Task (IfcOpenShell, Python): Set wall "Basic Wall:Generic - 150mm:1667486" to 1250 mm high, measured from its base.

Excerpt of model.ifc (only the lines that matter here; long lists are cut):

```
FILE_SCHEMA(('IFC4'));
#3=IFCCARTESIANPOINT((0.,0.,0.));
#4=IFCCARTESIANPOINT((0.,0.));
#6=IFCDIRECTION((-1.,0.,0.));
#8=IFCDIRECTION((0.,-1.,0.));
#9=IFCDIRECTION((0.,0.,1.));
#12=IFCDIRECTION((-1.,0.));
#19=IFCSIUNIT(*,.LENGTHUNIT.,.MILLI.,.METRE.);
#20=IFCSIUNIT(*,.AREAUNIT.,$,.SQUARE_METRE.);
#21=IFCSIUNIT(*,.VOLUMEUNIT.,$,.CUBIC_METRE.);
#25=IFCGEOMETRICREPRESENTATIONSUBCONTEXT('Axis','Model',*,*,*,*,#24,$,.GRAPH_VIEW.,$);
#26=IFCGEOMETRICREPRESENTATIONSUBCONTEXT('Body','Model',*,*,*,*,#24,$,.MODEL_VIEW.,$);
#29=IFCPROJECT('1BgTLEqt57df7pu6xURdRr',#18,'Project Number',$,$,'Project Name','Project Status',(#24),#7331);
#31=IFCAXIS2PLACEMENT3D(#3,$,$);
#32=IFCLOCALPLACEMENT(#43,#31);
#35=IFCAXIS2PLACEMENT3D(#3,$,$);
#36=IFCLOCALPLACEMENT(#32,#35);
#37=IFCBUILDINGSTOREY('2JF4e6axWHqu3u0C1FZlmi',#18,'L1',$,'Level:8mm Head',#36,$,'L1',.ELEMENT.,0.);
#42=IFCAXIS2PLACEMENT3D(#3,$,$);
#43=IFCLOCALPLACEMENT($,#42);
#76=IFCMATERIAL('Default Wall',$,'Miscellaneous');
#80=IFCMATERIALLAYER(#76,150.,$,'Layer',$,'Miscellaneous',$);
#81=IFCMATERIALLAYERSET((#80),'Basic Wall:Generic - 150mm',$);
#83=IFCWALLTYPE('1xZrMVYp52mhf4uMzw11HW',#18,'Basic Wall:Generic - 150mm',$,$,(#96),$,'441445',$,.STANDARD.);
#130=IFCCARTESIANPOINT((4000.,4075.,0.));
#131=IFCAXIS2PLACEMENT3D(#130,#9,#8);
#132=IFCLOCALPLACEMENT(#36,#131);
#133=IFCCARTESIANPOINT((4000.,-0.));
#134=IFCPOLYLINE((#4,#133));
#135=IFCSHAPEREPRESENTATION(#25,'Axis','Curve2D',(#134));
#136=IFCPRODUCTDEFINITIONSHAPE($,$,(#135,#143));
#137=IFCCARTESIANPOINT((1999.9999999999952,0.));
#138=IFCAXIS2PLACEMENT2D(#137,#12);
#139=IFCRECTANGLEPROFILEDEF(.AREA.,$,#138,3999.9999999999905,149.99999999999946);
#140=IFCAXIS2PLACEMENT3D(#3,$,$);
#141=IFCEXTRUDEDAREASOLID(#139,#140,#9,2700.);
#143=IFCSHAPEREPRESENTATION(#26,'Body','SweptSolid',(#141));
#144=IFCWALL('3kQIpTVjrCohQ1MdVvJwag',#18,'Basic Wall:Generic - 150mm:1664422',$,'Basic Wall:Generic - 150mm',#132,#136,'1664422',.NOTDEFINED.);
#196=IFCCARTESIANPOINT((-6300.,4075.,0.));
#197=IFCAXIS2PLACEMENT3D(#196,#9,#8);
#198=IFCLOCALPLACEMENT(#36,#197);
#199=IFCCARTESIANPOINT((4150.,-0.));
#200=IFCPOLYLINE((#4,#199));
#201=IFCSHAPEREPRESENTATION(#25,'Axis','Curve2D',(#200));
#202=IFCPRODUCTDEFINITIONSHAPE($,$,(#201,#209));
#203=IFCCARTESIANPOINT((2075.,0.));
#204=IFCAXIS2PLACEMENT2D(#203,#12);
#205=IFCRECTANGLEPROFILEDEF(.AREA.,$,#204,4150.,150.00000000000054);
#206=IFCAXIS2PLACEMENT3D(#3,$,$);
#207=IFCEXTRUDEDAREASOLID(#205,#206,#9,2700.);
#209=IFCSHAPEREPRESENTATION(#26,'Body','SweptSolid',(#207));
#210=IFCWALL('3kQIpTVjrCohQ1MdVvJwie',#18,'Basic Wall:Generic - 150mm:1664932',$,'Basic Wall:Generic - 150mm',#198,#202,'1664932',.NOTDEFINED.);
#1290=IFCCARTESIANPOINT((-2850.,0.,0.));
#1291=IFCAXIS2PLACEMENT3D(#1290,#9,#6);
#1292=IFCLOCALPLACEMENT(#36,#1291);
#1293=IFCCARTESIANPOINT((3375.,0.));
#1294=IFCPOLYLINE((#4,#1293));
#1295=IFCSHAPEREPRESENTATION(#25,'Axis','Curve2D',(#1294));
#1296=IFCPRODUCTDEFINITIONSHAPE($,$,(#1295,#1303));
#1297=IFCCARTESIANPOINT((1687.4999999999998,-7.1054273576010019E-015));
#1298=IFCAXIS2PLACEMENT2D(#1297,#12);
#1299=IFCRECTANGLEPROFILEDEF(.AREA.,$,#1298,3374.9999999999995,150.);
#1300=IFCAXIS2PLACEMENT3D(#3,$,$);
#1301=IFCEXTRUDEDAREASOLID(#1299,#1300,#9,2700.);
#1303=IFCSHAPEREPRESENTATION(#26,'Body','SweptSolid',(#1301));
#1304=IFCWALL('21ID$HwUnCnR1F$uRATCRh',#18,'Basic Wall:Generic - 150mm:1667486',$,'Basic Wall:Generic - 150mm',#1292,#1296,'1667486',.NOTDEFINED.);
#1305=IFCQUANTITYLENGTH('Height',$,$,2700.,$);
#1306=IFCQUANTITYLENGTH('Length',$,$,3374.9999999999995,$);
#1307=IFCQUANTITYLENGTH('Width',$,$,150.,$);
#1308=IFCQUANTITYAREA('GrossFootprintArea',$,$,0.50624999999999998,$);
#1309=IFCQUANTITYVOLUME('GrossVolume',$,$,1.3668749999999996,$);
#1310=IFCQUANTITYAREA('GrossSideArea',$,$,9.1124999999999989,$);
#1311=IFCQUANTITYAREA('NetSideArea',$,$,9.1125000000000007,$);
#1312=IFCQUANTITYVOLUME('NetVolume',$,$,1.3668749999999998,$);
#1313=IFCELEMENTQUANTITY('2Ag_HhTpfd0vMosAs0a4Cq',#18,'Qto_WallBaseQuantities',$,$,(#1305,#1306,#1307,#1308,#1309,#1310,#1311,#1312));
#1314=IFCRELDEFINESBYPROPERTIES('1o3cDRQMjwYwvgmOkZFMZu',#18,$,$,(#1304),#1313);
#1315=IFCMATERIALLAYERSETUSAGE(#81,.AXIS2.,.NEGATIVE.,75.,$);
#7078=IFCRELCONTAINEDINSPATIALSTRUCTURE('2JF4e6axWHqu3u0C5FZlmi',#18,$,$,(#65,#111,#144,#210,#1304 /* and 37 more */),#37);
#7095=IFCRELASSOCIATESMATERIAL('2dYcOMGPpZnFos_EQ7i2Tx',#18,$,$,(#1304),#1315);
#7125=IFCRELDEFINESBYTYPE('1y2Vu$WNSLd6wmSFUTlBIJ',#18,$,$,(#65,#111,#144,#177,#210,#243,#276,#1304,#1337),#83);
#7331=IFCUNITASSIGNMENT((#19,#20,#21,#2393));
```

```python
import ifcopenshell
import ifcopenshell.api.pset
import ifcopenshell.geom
import ifcopenshell.util.element
import ifcopenshell.util.representation
import ifcopenshell.util.shape
import ifcopenshell.util.unit

model = ifcopenshell.open("model.ifc")
unit_scale = ifcopenshell.util.unit.calculate_unit_scale(model)
area_scale = ifcopenshell.util.unit.calculate_unit_scale(model, "AREAUNIT")
volume_scale = ifcopenshell.util.unit.calculate_unit_scale(model, "VOLUMEUNIT")
settings = ifcopenshell.geom.settings()


def volume(element):
    """Net volume in cubic metres, openings subtracted."""
    shape = ifcopenshell.geom.create_shape(settings, element)
    return ifcopenshell.util.shape.get_volume(shape.geometry)


wall = model.by_guid("21ID$HwUnCnR1F$uRATCRh")
before = volume(wall)

body = ifcopenshell.util.representation.get_representation(wall, "Model", "Body")
solid = body.Items[0]
old_height = solid.Depth
solid.Depth = 1250.0
after = volume(wall)
thickness = 0.15  # wall thickness in metres

# Update the stored height, areas and volumes.
qto = model.by_id(ifcopenshell.util.element.get_pset(wall, "Qto_WallBaseQuantities", should_inherit=False)["id"])
ifcopenshell.api.pset.edit_qto(model, qto=qto, properties={
    "Height": solid.Depth,
    "GrossVolume": ifcopenshell.util.element.get_pset(wall, "Qto_WallBaseQuantities", "GrossVolume") * solid.Depth / old_height,
    "GrossSideArea": ifcopenshell.util.element.get_pset(wall, "Qto_WallBaseQuantities", "GrossSideArea") * solid.Depth / old_height,
    "NetSideArea": after / thickness / area_scale,
    "NetVolume": after / volume_scale,
})

print(f"height {old_height:g} -> {solid.Depth:g}, volume {before:.3f} -> {after:.3f} m3")

model.write("model_edited.ifc")
```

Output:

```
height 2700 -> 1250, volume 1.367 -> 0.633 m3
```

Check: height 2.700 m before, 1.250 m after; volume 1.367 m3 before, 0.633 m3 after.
